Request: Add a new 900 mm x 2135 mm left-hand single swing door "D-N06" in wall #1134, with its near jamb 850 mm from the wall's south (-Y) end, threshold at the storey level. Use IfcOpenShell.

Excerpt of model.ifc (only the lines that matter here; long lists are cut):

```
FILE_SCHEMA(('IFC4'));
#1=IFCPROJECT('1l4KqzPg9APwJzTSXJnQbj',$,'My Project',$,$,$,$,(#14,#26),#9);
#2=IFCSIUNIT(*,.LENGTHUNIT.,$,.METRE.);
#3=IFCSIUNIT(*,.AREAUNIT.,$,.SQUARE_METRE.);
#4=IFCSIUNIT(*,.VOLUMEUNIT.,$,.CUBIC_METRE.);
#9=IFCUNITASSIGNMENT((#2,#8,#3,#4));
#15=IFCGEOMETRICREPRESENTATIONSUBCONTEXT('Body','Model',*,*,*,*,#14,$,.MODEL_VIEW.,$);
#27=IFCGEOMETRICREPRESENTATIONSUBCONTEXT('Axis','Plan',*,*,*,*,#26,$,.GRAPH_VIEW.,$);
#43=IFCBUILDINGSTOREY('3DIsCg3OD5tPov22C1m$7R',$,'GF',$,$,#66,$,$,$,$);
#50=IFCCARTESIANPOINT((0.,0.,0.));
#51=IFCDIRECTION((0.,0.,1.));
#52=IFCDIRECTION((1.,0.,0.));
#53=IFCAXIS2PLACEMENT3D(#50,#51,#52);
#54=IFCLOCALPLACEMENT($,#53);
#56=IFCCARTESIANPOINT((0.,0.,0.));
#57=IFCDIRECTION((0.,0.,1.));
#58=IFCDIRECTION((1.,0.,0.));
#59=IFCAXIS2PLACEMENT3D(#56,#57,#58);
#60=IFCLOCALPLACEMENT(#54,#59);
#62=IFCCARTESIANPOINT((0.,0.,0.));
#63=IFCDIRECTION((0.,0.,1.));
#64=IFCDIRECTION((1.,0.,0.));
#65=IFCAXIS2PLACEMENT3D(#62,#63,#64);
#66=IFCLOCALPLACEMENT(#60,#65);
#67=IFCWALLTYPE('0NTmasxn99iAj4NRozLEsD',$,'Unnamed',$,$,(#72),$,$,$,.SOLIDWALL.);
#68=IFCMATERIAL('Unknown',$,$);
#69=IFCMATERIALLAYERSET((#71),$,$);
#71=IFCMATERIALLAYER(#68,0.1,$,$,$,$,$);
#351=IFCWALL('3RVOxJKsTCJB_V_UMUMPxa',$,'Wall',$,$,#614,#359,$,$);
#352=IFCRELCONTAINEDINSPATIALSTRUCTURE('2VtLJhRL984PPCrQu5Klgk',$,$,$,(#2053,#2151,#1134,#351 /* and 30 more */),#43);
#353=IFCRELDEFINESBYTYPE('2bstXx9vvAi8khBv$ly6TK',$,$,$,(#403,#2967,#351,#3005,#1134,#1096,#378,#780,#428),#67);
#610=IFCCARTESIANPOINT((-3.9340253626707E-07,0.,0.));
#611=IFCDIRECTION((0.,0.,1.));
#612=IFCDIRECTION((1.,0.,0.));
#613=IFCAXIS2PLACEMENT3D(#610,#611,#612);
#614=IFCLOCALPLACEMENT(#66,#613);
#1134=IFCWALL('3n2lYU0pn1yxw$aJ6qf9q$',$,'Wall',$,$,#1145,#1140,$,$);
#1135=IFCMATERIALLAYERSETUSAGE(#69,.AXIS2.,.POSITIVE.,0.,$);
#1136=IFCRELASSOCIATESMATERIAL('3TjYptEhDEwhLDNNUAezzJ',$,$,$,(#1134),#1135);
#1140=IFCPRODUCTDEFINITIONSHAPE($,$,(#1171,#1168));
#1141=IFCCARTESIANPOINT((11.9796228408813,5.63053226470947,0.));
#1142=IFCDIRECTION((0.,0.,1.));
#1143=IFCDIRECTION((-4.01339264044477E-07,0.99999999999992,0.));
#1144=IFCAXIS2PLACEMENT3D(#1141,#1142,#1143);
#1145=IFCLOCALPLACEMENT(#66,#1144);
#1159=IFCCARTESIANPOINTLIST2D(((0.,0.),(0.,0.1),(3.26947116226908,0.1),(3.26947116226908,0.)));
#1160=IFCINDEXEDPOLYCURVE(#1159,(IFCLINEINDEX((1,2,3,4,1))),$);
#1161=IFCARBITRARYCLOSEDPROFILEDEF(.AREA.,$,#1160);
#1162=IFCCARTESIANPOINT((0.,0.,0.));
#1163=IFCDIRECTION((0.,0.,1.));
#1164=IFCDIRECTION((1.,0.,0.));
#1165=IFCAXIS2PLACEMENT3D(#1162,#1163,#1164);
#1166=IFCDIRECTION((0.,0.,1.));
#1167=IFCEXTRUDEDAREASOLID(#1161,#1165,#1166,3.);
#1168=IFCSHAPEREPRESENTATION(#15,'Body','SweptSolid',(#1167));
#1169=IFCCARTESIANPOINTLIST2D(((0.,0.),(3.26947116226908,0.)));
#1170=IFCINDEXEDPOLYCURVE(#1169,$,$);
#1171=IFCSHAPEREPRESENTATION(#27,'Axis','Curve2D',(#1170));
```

```python
import numpy as np
import ifcopenshell
import ifcopenshell.api.feature
import ifcopenshell.api.geometry
import ifcopenshell.api.root
import ifcopenshell.api.spatial
import ifcopenshell.geom
import ifcopenshell.util.element
import ifcopenshell.util.placement
import ifcopenshell.util.representation
import ifcopenshell.util.shape
import ifcopenshell.util.unit

model = ifcopenshell.open("model.ifc")
unit_scale = ifcopenshell.util.unit.calculate_unit_scale(model)
settings = ifcopenshell.geom.settings()


def volume(element):
    """Net volume in cubic metres, openings subtracted."""
    shape = ifcopenshell.geom.create_shape(settings, element)
    return ifcopenshell.util.shape.get_volume(shape.geometry)


wall = model.by_guid("3n2lYU0pn1yxw$aJ6qf9q$")
storey = ifcopenshell.util.element.get_container(wall, ifc_class="IfcBuildingStorey")
context = ifcopenshell.util.representation.get_context(model, "Model", "Body", "MODEL_VIEW")
before = volume(wall)

width, height, from_end, sill = 0.9, 2.135, 0.85, 0.0  # metres

# The wall runs along its own X axis, and the end named is its -X end.
wall_shape = ifcopenshell.geom.create_shape(settings, wall)
x, y, z = ifcopenshell.util.shape.get_vertices(wall_shape.geometry).T
start = x.min() + from_end
face, thickness = float(y.min()), float(y.max() - y.min())
wall_matrix = ifcopenshell.util.placement.get_local_placement(wall.ObjectPlacement)
level = ifcopenshell.util.placement.get_local_placement(storey.ObjectPlacement)[2, 3]


def in_wall(x, y):
    """Placement at x, y metres in the wall's axes, at sill height."""
    matrix = wall_matrix.copy()
    matrix[:, 3] = wall_matrix @ np.array([x / unit_scale, y / unit_scale, 0.0, 1.0])
    matrix[2, 3] = level + sill / unit_scale
    return matrix


# Opening: a box that overshoots both wall faces by 50 mm.
opening = ifcopenshell.api.root.create_entity(model, ifc_class="IfcOpeningElement", predefined_type="OPENING")
box = ifcopenshell.api.geometry.add_wall_representation(
    model, context=context, length=width, height=height, thickness=thickness + 0.1
)
ifcopenshell.api.geometry.assign_representation(model, product=opening, representation=box)
ifcopenshell.api.geometry.edit_object_placement(model, product=opening, matrix=in_wall(start, face - 0.05), is_si=False)
ifcopenshell.api.feature.add_feature(model, feature=opening, element=wall)

door = ifcopenshell.api.root.create_entity(model, ifc_class="IfcDoor", name="D-N06", predefined_type="DOOR")
door.OverallWidth, door.OverallHeight = width / unit_scale, height / unit_scale
door.OperationType = "SINGLE_SWING_LEFT"
body = ifcopenshell.api.geometry.add_door_representation(
    model,
    context=context,
    overall_width=door.OverallWidth,
    overall_height=door.OverallHeight,
    operation_type="SINGLE_SWING_LEFT",
    lining_properties={"LiningDepth": thickness / unit_scale, "ThresholdDepth": thickness / unit_scale},
)
ifcopenshell.api.geometry.assign_representation(model, product=door, representation=body)
ifcopenshell.api.spatial.assign_container(model, products=[door], relating_structure=storey)
ifcopenshell.api.feature.add_filling(model, opening=opening, element=door)

# The lining spans the wall, so the door starts at the wall face.
ifcopenshell.api.geometry.edit_object_placement(model, product=door, matrix=in_wall(start, face), is_si=False)

after = volume(wall)

print(f"wall volume {before:.3f} -> {after:.3f} m3")

model.write("model_rev.ifc")
```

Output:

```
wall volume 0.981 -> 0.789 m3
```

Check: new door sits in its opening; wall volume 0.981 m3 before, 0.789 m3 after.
